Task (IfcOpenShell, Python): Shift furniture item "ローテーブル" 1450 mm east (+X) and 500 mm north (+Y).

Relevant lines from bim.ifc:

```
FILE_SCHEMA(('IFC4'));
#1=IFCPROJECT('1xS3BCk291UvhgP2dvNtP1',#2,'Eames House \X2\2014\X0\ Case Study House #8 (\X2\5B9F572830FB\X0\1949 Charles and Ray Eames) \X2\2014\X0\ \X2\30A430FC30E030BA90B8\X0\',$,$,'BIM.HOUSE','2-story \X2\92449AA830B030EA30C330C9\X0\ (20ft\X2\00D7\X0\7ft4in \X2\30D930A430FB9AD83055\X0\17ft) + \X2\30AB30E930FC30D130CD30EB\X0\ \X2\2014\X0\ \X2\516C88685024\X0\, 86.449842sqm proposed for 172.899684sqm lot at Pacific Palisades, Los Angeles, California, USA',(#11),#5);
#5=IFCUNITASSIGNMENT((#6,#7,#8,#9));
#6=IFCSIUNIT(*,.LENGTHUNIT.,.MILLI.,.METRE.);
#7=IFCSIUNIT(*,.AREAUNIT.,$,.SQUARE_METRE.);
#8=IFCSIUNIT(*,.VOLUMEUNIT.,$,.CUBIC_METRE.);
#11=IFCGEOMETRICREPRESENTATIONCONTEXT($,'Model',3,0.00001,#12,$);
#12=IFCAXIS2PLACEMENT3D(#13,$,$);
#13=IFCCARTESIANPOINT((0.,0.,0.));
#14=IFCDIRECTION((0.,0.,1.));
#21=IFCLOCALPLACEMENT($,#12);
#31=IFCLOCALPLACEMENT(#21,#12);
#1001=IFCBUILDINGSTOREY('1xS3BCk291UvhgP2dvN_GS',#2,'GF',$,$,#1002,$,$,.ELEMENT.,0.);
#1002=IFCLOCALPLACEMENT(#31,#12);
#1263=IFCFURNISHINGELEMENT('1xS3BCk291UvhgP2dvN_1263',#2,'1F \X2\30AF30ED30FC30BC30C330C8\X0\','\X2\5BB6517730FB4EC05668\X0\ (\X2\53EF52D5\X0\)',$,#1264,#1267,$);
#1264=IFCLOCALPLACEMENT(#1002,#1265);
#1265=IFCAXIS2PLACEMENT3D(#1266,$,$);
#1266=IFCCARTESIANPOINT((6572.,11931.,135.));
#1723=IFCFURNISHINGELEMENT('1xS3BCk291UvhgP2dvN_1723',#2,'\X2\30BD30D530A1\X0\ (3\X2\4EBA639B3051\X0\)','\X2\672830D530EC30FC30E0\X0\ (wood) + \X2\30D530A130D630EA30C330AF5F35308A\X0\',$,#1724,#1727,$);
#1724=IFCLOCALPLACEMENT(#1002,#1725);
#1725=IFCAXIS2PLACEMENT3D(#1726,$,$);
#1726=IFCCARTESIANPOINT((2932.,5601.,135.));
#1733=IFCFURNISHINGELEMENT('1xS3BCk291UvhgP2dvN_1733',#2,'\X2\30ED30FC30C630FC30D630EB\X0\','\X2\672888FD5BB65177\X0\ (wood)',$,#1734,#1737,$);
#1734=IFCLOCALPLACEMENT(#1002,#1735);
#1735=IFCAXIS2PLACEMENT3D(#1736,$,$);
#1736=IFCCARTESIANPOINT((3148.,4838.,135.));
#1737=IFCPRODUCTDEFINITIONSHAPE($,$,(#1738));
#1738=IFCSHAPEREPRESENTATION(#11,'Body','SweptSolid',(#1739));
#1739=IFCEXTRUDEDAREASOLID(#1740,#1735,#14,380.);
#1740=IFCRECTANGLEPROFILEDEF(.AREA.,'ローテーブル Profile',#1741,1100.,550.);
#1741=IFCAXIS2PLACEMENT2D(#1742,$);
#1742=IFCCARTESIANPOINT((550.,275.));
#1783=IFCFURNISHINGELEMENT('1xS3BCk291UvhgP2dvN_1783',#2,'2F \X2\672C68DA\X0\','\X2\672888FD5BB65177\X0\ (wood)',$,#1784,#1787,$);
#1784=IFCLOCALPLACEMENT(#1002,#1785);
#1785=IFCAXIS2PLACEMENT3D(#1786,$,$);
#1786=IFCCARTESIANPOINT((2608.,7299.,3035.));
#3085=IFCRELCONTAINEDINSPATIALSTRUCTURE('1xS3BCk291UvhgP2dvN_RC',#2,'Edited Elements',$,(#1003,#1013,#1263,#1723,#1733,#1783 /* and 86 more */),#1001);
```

```python
import ifcopenshell
import ifcopenshell.api.geometry
import ifcopenshell.util.placement

model = ifcopenshell.open("bim.ifc")

item = model.by_guid("1xS3BCk291UvhgP2dvN_1733")
matrix = ifcopenshell.util.placement.get_local_placement(item.ObjectPlacement)
matrix[0, 3] += 1450.0
matrix[1, 3] += 500.0
ifcopenshell.api.geometry.edit_object_placement(model, product=item, matrix=matrix, is_si=False)

print(ifcopenshell.util.placement.get_local_placement(item.ObjectPlacement).round(3) + 0.0)

model.write("bim-out.ifc")
```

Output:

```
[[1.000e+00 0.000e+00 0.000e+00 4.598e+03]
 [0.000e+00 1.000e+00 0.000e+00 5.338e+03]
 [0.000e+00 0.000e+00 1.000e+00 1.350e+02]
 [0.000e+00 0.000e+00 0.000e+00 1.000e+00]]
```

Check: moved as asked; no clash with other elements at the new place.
